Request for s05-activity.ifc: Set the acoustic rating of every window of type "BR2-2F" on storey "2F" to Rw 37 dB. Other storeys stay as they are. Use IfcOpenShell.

First a look at what the model holds.

```python
import ifcopenshell
import ifcopenshell.util.element

model = ifcopenshell.open("s05-activity.ifc")
print(model.schema)
storey = next(s for s in model.by_type("IfcBuildingStorey") if s.Name == "2F")
windows = [e for e in ifcopenshell.util.element.get_decomposition(storey) if e.is_a("IfcWindow")]
seen = {}
for e in windows:
    element_type = ifcopenshell.util.element.get_type(e)
    key = (element_type.Name if element_type != e and element_type else None, ifcopenshell.util.element.get_pset(e, "Pset_WindowCommon", "AcousticRating"))
    seen[key] = seen.get(key, 0) + 1
for (name, value), count in sorted(seen.items(), key=str):
    print(count, "x", name, "|", value)
```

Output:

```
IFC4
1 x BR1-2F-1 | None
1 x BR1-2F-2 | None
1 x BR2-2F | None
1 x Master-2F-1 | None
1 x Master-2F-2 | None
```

```python
import ifcopenshell
import ifcopenshell.api.pset
import ifcopenshell.util.element

model = ifcopenshell.open("s05-activity.ifc")

storey = next(s for s in model.by_type("IfcBuildingStorey") if s.Name == "2F")
windows = [e for e in ifcopenshell.util.element.get_decomposition(storey) if e.is_a("IfcWindow")]

count = 0
for e in windows:
    element_type = ifcopenshell.util.element.get_type(e)
    if element_type in (None, e) or element_type.Name != "BR2-2F":
        continue
    # add_pset returns the element's existing set when there is one.
    pset = ifcopenshell.api.pset.add_pset(model, product=e, name="Pset_WindowCommon")
    ifcopenshell.api.pset.edit_pset(model, pset=pset, properties={"AcousticRating": "Rw 37 dB"})
    count += 1

print(count, "windows updated")

model.write("s05-activity-out.ifc")
```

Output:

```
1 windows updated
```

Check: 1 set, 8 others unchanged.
